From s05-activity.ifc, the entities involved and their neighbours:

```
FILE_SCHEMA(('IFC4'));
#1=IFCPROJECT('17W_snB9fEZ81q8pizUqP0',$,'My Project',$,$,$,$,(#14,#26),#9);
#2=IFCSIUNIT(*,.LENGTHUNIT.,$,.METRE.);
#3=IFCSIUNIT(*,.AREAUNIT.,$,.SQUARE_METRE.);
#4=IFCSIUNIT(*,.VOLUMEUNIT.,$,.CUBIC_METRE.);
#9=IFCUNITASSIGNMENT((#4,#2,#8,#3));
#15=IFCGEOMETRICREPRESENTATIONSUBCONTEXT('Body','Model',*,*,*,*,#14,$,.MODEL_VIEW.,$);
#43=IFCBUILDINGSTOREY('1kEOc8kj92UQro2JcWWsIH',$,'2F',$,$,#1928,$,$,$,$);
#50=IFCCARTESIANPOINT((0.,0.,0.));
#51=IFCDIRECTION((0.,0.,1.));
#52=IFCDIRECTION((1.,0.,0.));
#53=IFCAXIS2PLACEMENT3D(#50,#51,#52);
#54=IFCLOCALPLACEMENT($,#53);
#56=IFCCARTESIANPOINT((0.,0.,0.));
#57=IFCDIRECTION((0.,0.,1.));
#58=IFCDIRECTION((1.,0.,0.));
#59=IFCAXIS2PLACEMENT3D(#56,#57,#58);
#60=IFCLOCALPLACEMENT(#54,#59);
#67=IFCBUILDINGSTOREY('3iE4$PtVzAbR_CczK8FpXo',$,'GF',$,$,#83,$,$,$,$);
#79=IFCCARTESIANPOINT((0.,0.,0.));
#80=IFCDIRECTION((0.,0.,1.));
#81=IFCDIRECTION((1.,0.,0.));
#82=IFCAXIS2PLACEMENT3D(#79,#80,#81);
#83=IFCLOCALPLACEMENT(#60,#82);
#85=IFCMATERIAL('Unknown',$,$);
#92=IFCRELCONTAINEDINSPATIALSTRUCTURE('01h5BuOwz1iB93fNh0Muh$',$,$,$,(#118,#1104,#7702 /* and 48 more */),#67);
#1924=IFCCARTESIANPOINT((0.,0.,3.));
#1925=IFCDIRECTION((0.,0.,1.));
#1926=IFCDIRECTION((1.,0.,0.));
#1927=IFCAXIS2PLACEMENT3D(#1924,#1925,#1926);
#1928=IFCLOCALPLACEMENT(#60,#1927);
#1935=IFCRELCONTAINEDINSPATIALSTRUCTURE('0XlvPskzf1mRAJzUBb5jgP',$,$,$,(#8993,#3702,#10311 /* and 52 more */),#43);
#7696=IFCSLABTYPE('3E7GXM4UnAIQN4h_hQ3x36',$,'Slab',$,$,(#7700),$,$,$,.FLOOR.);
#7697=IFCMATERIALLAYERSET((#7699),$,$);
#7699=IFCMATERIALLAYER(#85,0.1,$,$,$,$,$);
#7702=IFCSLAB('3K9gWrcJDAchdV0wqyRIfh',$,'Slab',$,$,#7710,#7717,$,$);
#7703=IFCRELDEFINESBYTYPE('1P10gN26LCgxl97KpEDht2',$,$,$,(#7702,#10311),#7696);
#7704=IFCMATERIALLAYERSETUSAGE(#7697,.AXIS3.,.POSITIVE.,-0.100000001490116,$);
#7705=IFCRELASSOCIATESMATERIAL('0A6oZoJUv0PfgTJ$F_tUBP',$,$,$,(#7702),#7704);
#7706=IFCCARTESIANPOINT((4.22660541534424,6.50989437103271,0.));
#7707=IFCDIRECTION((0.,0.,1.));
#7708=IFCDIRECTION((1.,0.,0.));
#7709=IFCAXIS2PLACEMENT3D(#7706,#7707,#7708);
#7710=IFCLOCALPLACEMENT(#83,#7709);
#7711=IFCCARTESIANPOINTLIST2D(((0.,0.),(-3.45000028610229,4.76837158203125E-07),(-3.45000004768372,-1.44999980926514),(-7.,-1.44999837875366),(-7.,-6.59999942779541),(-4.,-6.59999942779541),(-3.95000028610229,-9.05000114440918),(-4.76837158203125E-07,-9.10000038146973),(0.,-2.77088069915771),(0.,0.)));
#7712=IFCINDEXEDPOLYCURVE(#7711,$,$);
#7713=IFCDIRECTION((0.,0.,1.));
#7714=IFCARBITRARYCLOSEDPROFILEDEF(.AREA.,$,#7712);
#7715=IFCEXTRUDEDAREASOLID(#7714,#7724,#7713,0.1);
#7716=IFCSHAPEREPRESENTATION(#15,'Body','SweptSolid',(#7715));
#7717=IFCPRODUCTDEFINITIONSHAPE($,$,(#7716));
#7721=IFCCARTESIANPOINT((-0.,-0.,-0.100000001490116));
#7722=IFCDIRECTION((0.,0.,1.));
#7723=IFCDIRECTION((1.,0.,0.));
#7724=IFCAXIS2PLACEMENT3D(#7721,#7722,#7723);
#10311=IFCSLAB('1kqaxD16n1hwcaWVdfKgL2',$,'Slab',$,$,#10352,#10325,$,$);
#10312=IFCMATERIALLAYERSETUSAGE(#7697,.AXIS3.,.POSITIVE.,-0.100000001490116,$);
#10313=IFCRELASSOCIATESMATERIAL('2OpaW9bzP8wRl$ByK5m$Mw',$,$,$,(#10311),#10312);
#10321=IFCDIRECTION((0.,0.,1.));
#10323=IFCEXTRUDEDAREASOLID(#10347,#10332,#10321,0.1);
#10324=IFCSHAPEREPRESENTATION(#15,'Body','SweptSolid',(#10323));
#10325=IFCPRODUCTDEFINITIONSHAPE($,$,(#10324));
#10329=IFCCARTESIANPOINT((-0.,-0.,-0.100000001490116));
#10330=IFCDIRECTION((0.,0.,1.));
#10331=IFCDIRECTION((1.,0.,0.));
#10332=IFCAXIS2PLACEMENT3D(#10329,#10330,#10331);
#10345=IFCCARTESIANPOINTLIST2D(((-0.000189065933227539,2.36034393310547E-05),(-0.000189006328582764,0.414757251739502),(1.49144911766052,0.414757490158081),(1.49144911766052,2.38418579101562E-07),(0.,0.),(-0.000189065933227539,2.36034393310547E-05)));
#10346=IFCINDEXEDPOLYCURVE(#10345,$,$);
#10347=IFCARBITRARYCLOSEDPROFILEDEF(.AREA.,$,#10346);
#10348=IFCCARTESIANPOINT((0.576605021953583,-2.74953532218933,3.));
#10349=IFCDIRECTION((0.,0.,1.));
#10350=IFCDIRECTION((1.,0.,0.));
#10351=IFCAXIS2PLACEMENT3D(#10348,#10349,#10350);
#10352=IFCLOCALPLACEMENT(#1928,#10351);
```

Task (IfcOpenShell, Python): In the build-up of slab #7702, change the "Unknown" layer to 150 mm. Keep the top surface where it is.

```python
import ifcopenshell
import ifcopenshell.util.element
import ifcopenshell.util.representation

model = ifcopenshell.open("s05-activity.ifc")

layer_set = model.by_id(7697)
layer = next(l for l in layer_set.MaterialLayers if l.Material and l.Material.Name == "Unknown")
change = 0.15 - layer.LayerThickness
layer.LayerThickness += change

# The layer set is shared, so every slab that uses it gets the new thickness.
slabs = [e for e in ifcopenshell.util.element.get_elements_by_material(model, layer_set) if e.is_a("IfcSlab")]
for slab in sorted(slabs, key=lambda e: e.id()):
    body = ifcopenshell.util.representation.get_representation(slab, "Model", "Body")
    solid = body.Items[0]
    old_depth = solid.Depth
    solid.Depth += change
    # Extruded upwards: lower the start of the extrusion so the top stays.
    x, y, z = solid.Position.Location.Coordinates
    solid.Position.Location = model.createIfcCartesianPoint((x, y, z - change))
    print(slab.id(), f"{old_depth:g} -> {solid.Depth:g}")

# The layers are counted up from the underside, which has moved.
for usage in {ifcopenshell.util.element.get_material(slab) for slab in slabs}:
    usage.OffsetFromReferenceLine -= change

model.write("s05-activity-out.ifc")
```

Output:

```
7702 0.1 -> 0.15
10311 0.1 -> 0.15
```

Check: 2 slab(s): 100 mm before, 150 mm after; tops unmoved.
